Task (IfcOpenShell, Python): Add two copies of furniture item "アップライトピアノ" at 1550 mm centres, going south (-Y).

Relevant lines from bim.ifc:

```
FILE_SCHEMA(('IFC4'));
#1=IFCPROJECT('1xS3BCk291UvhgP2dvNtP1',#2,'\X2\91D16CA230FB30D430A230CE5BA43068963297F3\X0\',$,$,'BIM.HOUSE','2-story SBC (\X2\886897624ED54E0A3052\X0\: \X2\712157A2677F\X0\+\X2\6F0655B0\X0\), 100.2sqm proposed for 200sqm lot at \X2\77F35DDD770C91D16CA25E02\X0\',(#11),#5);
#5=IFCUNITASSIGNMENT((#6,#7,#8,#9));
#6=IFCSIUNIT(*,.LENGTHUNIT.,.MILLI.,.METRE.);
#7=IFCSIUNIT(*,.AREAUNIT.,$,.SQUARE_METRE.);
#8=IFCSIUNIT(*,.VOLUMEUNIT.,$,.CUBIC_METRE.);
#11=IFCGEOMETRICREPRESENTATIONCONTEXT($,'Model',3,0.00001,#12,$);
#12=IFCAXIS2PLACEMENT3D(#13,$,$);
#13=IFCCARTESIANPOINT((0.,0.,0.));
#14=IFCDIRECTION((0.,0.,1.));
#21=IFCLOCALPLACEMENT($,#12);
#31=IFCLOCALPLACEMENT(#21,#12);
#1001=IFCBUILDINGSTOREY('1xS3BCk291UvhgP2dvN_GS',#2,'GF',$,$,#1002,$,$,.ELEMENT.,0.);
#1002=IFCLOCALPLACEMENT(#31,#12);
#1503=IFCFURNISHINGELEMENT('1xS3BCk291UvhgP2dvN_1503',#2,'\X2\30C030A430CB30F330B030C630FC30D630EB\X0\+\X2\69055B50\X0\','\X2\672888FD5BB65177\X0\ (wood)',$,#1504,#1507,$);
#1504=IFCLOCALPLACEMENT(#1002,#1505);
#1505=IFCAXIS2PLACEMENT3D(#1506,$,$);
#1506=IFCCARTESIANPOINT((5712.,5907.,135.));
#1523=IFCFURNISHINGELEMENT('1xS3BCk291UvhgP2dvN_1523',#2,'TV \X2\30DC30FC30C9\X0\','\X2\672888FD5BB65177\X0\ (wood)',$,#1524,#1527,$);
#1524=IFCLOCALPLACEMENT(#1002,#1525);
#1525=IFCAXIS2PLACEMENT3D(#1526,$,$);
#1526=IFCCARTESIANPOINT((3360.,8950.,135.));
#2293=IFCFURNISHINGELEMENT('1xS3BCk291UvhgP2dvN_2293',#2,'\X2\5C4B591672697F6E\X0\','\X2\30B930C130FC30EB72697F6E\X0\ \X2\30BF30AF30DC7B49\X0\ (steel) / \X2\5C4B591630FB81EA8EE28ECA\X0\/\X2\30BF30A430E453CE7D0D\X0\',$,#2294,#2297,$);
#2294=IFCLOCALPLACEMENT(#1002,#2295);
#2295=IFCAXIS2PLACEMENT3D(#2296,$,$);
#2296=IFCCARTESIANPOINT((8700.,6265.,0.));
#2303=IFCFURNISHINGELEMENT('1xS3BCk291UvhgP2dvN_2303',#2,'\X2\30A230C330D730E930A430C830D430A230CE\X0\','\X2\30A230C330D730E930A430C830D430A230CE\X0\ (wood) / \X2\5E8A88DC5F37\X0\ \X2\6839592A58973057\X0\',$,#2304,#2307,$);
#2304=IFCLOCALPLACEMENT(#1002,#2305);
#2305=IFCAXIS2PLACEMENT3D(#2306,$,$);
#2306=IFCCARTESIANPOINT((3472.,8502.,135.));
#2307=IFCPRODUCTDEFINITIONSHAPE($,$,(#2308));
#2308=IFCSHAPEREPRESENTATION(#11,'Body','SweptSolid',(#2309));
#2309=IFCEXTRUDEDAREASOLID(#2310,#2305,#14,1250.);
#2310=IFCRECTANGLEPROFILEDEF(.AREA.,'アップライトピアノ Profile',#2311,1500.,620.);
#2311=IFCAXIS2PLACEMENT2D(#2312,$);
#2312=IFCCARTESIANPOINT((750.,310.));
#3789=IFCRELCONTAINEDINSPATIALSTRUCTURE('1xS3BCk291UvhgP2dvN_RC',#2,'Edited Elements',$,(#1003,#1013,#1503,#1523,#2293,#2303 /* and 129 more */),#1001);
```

```python
import numpy as np
import ifcopenshell
import ifcopenshell.api.geometry
import ifcopenshell.api.root
import ifcopenshell.util.element
import ifcopenshell.util.placement
import ifcopenshell.util.unit

model = ifcopenshell.open("bim.ifc")
unit_scale = ifcopenshell.util.unit.calculate_unit_scale(model)


def reuse_history(source, copy):
    """copy_class also copies each property set's owner history, people and application; keep the originals."""
    for rel in copy.IsDefinedBy:
        if rel.is_a("IfcRelDefinesByProperties") and (history := rel.RelatingPropertyDefinition.OwnerHistory):
            rel.RelatingPropertyDefinition.OwnerHistory = source.OwnerHistory
            ifcopenshell.util.element.remove_deep2(model, history)


source = model.by_id(2303)
base = ifcopenshell.util.placement.get_local_placement(source.ObjectPlacement)
step = np.array([0.0, -1.0, 0.0]) * 1.55 / unit_scale

for i in range(1, 3):
    copy = ifcopenshell.api.root.copy_class(model, product=source)
    copy.Representation = ifcopenshell.util.element.copy_deep(
        model, source.Representation, exclude=["IfcGeometricRepresentationContext", "IfcRepresentationMap"]
    )
    reuse_history(source, copy)
    matrix = base.copy()
    matrix[:3, 3] += i * step
    print("added at", matrix[:3, 3].round(3) + 0.0)
    ifcopenshell.api.geometry.edit_object_placement(model, product=copy, matrix=matrix, is_si=False)

model.write("bim_rev.ifc")
```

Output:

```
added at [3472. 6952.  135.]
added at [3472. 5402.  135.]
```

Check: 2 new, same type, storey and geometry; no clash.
